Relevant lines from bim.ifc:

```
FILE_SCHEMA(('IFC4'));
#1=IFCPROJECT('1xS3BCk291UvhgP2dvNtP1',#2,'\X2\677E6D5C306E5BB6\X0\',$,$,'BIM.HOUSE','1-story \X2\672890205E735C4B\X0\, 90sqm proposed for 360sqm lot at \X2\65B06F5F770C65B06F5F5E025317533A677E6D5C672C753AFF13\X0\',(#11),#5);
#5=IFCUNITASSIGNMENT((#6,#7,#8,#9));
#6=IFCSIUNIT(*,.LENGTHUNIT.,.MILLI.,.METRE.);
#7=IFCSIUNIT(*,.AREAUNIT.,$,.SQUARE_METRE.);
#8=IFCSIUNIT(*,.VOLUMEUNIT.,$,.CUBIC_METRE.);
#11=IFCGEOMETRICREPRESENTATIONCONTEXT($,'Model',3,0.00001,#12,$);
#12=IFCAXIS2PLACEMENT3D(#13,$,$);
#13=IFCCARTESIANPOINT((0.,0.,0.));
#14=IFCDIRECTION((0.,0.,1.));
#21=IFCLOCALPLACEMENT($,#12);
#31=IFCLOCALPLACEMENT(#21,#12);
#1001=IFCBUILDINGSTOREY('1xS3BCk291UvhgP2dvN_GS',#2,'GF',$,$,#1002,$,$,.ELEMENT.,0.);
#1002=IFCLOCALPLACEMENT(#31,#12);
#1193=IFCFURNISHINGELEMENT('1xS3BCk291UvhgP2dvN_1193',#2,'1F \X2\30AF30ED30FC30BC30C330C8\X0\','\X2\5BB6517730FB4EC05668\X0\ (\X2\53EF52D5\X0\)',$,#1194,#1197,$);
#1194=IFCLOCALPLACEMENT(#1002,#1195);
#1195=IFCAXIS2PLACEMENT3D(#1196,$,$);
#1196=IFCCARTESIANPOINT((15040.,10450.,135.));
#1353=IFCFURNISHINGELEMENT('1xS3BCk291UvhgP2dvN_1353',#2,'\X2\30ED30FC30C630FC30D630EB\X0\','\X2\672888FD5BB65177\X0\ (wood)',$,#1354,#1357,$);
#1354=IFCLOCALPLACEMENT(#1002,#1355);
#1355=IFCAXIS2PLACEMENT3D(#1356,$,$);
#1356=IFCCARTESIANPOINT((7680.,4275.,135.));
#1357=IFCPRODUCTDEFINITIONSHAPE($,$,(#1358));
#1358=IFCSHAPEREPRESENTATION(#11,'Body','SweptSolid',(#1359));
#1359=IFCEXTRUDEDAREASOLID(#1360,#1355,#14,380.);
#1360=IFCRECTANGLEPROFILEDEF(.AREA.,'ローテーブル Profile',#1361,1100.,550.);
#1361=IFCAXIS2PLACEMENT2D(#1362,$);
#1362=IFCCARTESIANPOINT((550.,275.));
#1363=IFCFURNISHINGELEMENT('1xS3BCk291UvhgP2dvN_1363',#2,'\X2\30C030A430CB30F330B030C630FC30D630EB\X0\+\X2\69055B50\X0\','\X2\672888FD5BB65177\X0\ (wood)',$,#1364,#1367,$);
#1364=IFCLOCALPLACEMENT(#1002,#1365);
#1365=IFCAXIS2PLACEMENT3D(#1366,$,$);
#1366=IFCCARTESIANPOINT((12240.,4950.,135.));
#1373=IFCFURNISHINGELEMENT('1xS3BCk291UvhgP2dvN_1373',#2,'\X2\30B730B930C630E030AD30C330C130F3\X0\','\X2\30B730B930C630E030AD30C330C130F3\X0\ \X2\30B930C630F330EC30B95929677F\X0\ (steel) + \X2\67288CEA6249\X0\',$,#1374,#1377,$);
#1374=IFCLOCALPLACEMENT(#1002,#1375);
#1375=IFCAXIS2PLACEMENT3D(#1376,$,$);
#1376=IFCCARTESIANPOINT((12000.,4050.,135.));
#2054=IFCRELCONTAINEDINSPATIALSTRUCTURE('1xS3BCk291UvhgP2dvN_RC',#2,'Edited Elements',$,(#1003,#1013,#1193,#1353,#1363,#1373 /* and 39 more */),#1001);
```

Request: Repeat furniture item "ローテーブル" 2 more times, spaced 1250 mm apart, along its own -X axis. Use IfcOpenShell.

```python
import ifcopenshell
import ifcopenshell.api.geometry
import ifcopenshell.api.root
import ifcopenshell.util.element
import ifcopenshell.util.placement

model = ifcopenshell.open("bim.ifc")


def reuse_history(source, copy):
    """copy_class also copies each property set's owner history, people and application; keep the originals."""
    for rel in copy.IsDefinedBy:
        if rel.is_a("IfcRelDefinesByProperties") and (history := rel.RelatingPropertyDefinition.OwnerHistory):
            rel.RelatingPropertyDefinition.OwnerHistory = source.OwnerHistory
            ifcopenshell.util.element.remove_deep2(model, history)


source = model.by_guid("1xS3BCk291UvhgP2dvN_1353")
base = ifcopenshell.util.placement.get_local_placement(source.ObjectPlacement)
step = -base[:3, 0] * 1250.0

for i in range(1, 3):
    copy = ifcopenshell.api.root.copy_class(model, product=source)
    copy.Representation = ifcopenshell.util.element.copy_deep(
        model, source.Representation, exclude=["IfcGeometricRepresentationContext", "IfcRepresentationMap"]
    )
    reuse_history(source, copy)
    matrix = base.copy()
    matrix[:3, 3] += i * step
    print("added at", matrix[:3, 3].round(3) + 0.0)
    ifcopenshell.api.geometry.edit_object_placement(model, product=copy, matrix=matrix, is_si=False)

model.write("bim_edited.ifc")
```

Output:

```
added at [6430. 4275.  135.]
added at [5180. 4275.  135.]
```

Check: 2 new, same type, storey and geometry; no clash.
